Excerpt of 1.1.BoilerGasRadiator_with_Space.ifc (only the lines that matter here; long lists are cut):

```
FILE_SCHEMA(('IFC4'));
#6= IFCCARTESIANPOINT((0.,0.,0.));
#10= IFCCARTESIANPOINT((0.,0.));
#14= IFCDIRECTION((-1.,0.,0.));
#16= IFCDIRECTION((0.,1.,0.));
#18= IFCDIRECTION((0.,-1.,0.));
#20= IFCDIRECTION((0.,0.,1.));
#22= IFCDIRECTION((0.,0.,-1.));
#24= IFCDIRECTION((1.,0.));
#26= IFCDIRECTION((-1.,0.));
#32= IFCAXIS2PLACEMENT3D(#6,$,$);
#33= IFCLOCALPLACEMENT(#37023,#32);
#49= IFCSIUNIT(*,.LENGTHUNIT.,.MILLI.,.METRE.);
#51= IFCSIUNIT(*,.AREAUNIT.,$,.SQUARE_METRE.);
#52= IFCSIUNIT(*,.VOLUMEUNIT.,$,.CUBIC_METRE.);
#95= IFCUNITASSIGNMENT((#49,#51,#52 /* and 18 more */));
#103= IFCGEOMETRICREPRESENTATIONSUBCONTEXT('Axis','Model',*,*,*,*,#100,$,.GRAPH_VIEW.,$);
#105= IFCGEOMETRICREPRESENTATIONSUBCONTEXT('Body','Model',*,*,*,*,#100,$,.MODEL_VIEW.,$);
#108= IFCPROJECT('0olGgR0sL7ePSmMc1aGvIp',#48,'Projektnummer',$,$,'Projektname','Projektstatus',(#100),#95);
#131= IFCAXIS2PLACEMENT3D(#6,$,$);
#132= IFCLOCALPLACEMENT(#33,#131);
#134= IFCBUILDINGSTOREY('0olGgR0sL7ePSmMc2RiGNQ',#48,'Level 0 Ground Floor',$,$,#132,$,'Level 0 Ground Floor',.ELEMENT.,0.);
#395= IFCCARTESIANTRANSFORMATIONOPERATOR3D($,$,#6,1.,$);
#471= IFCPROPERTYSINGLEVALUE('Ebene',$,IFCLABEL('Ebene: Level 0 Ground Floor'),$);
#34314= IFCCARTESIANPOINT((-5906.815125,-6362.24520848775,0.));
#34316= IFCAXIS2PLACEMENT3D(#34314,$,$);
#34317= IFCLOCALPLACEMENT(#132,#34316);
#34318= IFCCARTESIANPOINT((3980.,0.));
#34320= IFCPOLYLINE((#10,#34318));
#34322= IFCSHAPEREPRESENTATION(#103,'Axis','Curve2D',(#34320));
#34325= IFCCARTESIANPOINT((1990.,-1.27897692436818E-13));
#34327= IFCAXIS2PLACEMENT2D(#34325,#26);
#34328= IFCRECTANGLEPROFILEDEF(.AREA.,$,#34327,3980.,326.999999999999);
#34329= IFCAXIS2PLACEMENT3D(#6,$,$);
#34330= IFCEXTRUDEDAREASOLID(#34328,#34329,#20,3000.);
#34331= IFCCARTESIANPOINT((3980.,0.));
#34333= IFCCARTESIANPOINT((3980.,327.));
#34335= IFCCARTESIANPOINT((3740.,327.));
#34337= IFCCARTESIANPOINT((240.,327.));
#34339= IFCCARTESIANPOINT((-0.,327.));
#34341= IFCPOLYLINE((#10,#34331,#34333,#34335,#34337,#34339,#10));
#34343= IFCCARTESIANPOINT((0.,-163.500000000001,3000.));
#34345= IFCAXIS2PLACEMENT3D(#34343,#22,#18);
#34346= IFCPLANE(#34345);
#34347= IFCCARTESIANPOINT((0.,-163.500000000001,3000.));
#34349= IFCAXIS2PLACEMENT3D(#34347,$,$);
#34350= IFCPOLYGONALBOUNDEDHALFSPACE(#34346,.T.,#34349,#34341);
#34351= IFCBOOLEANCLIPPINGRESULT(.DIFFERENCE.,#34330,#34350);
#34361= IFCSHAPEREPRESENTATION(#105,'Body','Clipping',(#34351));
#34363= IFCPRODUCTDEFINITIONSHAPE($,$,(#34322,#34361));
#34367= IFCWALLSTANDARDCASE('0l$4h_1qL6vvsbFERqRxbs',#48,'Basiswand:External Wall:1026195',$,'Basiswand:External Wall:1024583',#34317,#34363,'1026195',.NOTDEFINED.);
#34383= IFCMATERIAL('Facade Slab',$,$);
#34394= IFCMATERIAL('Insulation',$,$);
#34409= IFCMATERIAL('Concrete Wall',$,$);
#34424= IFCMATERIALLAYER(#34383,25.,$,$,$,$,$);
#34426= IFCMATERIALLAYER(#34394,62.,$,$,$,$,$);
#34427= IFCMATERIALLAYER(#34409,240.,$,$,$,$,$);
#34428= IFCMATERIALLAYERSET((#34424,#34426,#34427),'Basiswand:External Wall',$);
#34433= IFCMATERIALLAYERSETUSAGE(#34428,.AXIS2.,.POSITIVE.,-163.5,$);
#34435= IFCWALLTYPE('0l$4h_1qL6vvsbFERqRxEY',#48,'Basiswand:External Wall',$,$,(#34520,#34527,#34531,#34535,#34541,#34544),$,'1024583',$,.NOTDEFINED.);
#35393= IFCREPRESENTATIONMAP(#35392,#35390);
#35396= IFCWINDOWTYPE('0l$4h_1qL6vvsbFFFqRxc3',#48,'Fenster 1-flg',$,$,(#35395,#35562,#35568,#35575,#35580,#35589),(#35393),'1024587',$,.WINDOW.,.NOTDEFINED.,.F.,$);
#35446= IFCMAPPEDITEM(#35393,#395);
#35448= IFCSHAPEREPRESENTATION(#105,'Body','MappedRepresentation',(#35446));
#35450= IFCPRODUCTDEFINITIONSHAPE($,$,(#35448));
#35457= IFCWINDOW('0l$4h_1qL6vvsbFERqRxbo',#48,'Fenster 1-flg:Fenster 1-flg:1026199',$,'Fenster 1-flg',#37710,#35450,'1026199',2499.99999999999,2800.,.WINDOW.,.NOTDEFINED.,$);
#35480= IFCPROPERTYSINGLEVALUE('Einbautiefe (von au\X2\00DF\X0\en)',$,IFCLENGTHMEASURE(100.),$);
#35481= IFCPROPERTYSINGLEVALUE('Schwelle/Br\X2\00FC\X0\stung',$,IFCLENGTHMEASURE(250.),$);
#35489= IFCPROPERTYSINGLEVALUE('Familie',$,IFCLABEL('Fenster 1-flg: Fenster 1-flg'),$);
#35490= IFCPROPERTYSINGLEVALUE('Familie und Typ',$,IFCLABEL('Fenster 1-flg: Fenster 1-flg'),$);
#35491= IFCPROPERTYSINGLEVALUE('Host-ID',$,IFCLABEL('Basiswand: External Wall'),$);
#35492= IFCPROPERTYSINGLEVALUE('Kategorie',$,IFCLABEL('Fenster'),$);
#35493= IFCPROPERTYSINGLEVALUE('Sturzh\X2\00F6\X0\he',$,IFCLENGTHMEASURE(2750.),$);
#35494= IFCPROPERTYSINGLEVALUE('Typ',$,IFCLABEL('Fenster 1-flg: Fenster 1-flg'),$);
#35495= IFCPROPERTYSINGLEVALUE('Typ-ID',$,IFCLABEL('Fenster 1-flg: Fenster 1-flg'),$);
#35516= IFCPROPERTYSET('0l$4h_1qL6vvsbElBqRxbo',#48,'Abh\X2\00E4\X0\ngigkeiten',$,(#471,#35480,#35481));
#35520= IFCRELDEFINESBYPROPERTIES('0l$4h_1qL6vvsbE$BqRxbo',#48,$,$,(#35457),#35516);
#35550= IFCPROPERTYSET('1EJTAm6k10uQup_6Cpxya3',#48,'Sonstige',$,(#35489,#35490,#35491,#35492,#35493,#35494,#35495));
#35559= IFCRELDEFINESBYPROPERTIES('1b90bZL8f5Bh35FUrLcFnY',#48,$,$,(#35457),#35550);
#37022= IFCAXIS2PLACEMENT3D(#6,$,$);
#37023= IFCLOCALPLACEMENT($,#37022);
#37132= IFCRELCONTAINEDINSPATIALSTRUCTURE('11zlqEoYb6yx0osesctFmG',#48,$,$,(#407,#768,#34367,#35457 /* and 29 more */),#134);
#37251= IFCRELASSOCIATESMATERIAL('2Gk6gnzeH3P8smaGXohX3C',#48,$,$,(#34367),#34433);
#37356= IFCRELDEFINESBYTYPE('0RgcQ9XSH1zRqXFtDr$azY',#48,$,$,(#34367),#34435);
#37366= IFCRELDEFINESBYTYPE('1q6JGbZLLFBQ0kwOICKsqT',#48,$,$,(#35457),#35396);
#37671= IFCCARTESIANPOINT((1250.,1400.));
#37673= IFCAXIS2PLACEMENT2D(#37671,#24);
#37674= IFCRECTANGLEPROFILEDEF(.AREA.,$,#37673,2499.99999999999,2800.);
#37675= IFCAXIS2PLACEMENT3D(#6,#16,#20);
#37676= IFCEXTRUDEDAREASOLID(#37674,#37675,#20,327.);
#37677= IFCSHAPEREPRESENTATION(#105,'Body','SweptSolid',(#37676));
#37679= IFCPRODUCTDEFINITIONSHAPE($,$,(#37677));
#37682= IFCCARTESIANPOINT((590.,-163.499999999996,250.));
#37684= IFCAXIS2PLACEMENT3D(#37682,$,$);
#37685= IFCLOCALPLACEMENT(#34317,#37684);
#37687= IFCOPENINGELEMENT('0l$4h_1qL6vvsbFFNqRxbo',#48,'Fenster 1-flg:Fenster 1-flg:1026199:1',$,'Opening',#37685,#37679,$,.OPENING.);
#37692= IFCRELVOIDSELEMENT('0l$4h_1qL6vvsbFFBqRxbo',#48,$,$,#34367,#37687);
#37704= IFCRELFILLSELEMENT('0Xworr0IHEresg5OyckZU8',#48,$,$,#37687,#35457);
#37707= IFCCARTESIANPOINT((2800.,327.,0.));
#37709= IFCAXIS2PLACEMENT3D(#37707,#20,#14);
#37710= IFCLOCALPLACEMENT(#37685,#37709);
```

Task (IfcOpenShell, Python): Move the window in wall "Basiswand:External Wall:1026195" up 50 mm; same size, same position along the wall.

```python
import numpy as np
import ifcopenshell
import ifcopenshell.api.geometry
import ifcopenshell.api.pset
import ifcopenshell.util.element
import ifcopenshell.util.placement
import ifcopenshell.util.unit

model = ifcopenshell.open("1.1.BoilerGasRadiator_with_Space.ifc")
unit_scale = ifcopenshell.util.unit.calculate_unit_scale(model)

window = model.by_id(35457)
opening = window.FillsVoids[0].RelatingOpeningElement
dz = 0.05 / unit_scale

shift = np.array([0.0, 0.0, dz])
# The window is placed relative to its opening, so it follows when the opening moves.
matrix = ifcopenshell.util.placement.get_local_placement(opening.ObjectPlacement)
matrix[:3, 3] += shift
ifcopenshell.api.geometry.edit_object_placement(
    model, product=opening, matrix=matrix, is_si=False, should_transform_children=True
)

# Keep the stored heights in step.
pset = model.by_id(ifcopenshell.util.element.get_pset(window, "Abhängigkeiten", should_inherit=False)["id"])
ifcopenshell.api.pset.edit_pset(model, pset=pset, properties={
    "Schwelle/Brüstung": model.create_entity("IfcLengthMeasure", ifcopenshell.util.element.get_pset(window, "Abhängigkeiten", "Schwelle/Brüstung") + dz),
})
pset = model.by_id(ifcopenshell.util.element.get_pset(window, "Sonstige", should_inherit=False)["id"])
ifcopenshell.api.pset.edit_pset(model, pset=pset, properties={
    "Sturzhöhe": model.create_entity("IfcLengthMeasure", ifcopenshell.util.element.get_pset(window, "Sonstige", "Sturzhöhe") + dz),
})

print(f"moved by {dz * unit_scale:+.3f} m")

model.write("1.1.BoilerGasRadiator_with_Space-out.ifc")
```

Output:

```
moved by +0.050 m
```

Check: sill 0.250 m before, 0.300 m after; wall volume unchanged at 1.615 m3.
